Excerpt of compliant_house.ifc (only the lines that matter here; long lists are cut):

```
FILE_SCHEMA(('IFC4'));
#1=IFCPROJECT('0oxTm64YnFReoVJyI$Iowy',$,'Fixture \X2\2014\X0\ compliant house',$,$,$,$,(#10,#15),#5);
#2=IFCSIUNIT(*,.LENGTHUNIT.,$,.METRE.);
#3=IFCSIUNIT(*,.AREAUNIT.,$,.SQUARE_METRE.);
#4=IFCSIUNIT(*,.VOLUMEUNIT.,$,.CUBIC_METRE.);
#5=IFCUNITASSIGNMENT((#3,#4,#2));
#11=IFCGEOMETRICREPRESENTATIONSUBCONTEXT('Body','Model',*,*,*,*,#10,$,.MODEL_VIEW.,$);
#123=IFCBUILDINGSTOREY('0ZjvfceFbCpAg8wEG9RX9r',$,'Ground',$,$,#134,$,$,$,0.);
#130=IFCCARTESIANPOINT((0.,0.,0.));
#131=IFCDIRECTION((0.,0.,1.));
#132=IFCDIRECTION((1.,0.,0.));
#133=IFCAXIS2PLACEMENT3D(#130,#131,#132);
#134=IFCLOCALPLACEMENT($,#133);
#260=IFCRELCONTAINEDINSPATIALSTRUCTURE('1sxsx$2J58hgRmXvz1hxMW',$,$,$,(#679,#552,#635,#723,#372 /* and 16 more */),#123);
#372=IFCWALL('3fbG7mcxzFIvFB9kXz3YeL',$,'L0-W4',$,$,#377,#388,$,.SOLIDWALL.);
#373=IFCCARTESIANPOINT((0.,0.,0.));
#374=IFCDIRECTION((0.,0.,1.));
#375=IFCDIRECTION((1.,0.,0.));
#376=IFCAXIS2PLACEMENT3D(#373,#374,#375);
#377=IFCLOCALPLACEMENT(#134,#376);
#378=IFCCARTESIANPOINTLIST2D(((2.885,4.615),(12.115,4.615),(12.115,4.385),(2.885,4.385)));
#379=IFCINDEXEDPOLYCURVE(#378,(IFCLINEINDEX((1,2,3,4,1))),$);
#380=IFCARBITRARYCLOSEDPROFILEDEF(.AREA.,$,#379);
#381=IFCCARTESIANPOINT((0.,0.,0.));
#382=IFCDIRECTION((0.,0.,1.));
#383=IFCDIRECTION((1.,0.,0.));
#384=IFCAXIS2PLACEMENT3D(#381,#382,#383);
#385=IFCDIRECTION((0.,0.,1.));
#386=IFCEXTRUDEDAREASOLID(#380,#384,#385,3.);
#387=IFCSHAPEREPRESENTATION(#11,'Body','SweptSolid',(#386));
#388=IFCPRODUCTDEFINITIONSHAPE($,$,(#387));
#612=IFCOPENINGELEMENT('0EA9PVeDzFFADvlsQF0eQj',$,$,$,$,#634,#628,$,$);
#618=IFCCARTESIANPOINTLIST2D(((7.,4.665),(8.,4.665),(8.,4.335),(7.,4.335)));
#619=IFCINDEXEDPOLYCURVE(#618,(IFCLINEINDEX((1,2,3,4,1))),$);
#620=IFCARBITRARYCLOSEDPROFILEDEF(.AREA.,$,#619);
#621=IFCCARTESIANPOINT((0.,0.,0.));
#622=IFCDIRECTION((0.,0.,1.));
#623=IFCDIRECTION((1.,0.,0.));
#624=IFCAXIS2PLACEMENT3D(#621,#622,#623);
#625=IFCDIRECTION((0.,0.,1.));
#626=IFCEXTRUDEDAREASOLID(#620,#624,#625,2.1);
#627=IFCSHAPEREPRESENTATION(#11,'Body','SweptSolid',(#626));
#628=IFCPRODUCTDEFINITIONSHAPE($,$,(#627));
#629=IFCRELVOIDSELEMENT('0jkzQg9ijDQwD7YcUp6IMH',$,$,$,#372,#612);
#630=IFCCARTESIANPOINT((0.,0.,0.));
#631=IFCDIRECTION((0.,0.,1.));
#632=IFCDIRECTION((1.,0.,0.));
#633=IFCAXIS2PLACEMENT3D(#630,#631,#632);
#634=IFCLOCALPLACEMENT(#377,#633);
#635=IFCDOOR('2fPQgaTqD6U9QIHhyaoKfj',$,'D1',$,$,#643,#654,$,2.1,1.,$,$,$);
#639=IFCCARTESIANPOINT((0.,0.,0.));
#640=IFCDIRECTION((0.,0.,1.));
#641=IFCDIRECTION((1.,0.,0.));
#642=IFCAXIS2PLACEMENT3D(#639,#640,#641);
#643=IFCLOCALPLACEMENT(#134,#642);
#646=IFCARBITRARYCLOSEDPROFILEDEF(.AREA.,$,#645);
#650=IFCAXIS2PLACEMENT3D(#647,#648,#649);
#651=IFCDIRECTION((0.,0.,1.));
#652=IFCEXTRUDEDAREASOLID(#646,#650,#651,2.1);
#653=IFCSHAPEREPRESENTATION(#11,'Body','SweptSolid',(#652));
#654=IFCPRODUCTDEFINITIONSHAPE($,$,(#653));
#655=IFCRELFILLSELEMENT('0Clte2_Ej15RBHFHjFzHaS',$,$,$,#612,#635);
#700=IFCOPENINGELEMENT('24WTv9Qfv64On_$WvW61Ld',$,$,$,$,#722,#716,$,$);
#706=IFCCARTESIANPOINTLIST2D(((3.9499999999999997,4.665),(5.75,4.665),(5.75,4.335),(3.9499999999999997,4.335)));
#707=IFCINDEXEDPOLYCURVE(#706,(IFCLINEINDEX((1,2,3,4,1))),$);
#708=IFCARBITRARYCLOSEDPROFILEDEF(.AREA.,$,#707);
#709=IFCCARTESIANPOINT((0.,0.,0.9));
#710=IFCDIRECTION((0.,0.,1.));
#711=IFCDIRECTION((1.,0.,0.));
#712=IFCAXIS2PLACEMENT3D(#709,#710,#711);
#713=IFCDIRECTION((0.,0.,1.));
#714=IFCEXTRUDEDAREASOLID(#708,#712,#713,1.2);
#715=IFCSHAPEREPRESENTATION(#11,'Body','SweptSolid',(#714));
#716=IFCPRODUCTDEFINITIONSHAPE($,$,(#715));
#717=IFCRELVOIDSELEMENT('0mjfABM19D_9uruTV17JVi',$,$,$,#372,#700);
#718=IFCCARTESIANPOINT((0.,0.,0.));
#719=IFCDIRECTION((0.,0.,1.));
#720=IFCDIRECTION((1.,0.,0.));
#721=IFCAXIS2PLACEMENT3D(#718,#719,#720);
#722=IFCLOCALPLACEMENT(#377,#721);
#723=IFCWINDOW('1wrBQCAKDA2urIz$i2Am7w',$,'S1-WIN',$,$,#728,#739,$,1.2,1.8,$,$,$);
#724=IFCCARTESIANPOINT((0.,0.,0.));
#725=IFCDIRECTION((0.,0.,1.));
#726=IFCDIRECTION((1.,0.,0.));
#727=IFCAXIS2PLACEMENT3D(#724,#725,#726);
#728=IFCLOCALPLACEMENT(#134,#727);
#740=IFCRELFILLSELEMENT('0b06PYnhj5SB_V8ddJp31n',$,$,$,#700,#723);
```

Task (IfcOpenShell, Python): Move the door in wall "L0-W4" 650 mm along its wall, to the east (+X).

```python
import ifcopenshell
import ifcopenshell.api.geometry
import ifcopenshell.util.placement
import ifcopenshell.util.unit

model = ifcopenshell.open("compliant_house.ifc")
unit_scale = ifcopenshell.util.unit.calculate_unit_scale(model)

door = model.by_id(635)
opening = door.FillsVoids[0].RelatingOpeningElement
wall = opening.VoidsElements[0].RelatingBuildingElement

wall_matrix = ifcopenshell.util.placement.get_local_placement(wall.ObjectPlacement)
shift = wall_matrix[:3, 0] * 0.65 / unit_scale
before = ifcopenshell.util.placement.get_local_placement(door.ObjectPlacement)[:3, 3].copy()

# The door is not placed relative to its opening, so move both.
for product in (opening, door):
    matrix = ifcopenshell.util.placement.get_local_placement(product.ObjectPlacement)
    matrix[:3, 3] += shift
    ifcopenshell.api.geometry.edit_object_placement(model, product=product, matrix=matrix, is_si=False)

after = ifcopenshell.util.placement.get_local_placement(door.ObjectPlacement)[:3, 3]
print("door moved by", (after - before).round(3) + 0.0)

model.write("compliant_house_v2.ifc")
```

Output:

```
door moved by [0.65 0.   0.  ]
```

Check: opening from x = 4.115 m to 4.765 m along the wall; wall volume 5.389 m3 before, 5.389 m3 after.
